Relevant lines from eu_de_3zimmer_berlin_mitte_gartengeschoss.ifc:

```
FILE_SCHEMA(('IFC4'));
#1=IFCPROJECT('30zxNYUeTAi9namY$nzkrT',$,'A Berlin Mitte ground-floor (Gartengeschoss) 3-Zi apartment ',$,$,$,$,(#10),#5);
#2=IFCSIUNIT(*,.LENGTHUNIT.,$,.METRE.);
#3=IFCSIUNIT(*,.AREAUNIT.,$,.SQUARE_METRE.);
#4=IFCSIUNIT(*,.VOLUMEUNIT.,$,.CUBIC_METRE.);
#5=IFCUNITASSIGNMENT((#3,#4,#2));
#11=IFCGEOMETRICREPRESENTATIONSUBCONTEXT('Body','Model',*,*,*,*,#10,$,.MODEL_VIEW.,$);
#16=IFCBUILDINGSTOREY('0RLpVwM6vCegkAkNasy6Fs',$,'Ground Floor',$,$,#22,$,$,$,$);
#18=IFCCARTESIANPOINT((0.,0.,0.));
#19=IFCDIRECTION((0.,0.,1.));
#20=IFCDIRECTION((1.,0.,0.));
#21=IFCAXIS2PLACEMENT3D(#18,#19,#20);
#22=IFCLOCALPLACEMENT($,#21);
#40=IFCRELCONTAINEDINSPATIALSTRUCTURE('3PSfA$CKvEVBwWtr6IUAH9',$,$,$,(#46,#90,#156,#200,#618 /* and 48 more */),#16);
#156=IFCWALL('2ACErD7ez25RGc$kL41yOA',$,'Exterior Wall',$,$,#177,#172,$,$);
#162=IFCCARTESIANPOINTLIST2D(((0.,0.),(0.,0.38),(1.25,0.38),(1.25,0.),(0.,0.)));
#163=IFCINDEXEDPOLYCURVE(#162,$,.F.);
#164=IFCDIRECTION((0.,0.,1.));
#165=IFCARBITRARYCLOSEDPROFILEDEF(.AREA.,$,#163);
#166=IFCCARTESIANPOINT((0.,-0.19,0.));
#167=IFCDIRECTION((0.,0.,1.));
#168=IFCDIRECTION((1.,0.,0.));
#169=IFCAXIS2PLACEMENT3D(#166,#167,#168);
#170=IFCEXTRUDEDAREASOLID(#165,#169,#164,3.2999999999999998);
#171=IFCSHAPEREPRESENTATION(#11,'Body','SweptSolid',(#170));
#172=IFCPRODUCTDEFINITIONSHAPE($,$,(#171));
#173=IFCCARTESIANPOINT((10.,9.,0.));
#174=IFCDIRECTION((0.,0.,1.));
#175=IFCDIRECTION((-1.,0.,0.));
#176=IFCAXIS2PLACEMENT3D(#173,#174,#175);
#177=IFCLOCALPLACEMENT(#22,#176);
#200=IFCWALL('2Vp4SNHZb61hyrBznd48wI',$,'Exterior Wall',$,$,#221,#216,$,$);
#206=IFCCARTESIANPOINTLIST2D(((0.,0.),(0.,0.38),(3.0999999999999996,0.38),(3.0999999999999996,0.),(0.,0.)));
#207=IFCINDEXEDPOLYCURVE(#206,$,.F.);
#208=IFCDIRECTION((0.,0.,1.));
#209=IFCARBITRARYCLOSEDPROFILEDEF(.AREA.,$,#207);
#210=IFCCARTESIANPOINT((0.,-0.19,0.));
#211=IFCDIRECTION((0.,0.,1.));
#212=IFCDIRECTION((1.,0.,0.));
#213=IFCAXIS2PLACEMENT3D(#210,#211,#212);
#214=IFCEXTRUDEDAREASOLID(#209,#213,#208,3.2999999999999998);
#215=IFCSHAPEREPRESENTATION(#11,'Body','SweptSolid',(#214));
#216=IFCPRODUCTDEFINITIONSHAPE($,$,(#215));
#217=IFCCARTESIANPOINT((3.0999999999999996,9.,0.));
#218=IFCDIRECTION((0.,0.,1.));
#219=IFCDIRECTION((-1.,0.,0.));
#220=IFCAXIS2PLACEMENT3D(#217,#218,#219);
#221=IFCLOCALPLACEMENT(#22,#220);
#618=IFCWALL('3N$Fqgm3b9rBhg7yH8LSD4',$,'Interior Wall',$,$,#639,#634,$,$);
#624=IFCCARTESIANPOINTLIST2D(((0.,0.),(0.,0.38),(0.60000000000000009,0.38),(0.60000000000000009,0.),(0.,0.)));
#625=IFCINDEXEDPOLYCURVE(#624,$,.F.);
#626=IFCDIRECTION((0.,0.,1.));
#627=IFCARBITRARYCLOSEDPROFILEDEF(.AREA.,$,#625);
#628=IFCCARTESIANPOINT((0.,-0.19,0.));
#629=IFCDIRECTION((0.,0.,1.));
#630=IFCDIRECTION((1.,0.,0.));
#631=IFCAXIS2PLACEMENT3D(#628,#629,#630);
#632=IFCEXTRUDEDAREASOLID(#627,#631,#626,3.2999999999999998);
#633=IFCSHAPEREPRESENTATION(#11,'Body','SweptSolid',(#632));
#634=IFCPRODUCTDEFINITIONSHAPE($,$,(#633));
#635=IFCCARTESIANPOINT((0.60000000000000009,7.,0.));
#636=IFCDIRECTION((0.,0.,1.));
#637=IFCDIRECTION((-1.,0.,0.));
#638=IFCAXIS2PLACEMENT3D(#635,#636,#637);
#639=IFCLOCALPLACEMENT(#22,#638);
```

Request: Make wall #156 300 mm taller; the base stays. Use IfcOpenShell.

```python
import ifcopenshell
import ifcopenshell.geom
import ifcopenshell.util.representation
import ifcopenshell.util.shape
import ifcopenshell.util.unit

model = ifcopenshell.open("eu_de_3zimmer_berlin_mitte_gartengeschoss.ifc")
unit_scale = ifcopenshell.util.unit.calculate_unit_scale(model)
settings = ifcopenshell.geom.settings()


def volume(element):
    """Net volume in cubic metres, openings subtracted."""
    shape = ifcopenshell.geom.create_shape(settings, element)
    return ifcopenshell.util.shape.get_volume(shape.geometry)


wall = model.by_guid("2ACErD7ez25RGc$kL41yOA")
before = volume(wall)

body = ifcopenshell.util.representation.get_representation(wall, "Model", "Body")
solid = body.Items[0]
old_height = solid.Depth
solid.Depth += 0.3 / unit_scale
after = volume(wall)

print(f"height {old_height:g} -> {solid.Depth:g}, volume {before:.3f} -> {after:.3f} m3")

model.write("eu_de_3zimmer_berlin_mitte_gartengeschoss_edited.ifc")
```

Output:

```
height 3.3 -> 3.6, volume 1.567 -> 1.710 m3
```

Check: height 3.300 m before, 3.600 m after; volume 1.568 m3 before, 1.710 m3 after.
